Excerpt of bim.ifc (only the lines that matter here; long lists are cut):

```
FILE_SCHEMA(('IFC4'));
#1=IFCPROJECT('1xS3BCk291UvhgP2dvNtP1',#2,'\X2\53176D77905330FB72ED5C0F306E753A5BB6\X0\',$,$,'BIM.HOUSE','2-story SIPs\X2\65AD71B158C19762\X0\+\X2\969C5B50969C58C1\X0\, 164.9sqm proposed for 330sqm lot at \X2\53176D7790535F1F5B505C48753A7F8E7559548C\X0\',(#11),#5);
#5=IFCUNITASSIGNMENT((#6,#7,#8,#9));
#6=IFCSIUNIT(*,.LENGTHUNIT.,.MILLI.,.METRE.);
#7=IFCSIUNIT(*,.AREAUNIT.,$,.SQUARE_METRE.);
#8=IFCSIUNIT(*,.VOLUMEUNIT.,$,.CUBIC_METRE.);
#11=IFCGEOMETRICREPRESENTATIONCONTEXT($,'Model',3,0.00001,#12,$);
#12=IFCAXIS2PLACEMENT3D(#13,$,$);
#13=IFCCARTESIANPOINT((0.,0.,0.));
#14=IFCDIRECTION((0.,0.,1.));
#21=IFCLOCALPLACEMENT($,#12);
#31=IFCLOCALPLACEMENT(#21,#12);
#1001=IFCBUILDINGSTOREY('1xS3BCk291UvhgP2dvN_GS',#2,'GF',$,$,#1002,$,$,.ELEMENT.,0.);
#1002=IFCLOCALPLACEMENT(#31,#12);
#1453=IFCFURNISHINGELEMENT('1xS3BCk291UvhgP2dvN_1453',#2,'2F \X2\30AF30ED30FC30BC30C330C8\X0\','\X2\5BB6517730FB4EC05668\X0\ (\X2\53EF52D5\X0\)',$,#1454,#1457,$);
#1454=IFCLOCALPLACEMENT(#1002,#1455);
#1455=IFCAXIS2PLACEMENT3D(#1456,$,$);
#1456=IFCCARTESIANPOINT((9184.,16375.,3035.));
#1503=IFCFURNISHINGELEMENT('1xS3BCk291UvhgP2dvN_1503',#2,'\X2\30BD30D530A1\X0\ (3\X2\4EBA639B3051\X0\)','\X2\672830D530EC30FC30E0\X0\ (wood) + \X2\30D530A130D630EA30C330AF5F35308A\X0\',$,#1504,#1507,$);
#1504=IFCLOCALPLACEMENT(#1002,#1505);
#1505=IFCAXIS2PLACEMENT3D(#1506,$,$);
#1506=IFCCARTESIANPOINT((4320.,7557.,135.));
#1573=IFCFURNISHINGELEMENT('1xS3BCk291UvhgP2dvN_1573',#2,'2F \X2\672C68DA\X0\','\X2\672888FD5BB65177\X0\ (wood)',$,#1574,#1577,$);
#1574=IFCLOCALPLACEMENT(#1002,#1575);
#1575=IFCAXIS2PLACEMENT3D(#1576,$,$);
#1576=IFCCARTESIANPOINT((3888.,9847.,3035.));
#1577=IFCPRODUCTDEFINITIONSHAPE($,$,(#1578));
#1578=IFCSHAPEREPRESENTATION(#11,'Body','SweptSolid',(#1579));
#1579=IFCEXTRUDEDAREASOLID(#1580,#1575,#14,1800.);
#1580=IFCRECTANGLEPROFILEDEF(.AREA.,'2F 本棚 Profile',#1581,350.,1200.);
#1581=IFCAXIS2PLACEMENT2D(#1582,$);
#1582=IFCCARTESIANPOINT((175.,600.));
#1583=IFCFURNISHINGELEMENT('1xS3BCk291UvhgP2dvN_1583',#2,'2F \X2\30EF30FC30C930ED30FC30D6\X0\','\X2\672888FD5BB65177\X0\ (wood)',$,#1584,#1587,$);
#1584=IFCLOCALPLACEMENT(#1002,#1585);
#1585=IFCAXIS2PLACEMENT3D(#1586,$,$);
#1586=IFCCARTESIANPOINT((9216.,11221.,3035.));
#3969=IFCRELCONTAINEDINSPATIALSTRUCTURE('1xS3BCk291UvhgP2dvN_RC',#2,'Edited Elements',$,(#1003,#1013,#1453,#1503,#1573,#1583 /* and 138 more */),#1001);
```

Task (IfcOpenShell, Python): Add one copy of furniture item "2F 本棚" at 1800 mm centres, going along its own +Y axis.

```python
import ifcopenshell
import ifcopenshell.api.geometry
import ifcopenshell.api.root
import ifcopenshell.util.element
import ifcopenshell.util.placement

model = ifcopenshell.open("bim.ifc")


def reuse_history(source, copy):
    """copy_class also copies each property set's owner history, people and application; keep the originals."""
    for rel in copy.IsDefinedBy:
        if rel.is_a("IfcRelDefinesByProperties") and (history := rel.RelatingPropertyDefinition.OwnerHistory):
            rel.RelatingPropertyDefinition.OwnerHistory = source.OwnerHistory
            ifcopenshell.util.element.remove_deep2(model, history)


source = model.by_guid("1xS3BCk291UvhgP2dvN_1573")
base = ifcopenshell.util.placement.get_local_placement(source.ObjectPlacement)
step = base[:3, 1] * 1800.0

for i in range(1, 2):
    copy = ifcopenshell.api.root.copy_class(model, product=source)
    copy.Representation = ifcopenshell.util.element.copy_deep(
        model, source.Representation, exclude=["IfcGeometricRepresentationContext", "IfcRepresentationMap"]
    )
    reuse_history(source, copy)
    matrix = base.copy()
    matrix[:3, 3] += i * step
    print("added at", matrix[:3, 3].round(3) + 0.0)
    ifcopenshell.api.geometry.edit_object_placement(model, product=copy, matrix=matrix, is_si=False)

model.write("bim_v2.ifc")
```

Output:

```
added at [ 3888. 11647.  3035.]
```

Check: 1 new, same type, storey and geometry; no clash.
